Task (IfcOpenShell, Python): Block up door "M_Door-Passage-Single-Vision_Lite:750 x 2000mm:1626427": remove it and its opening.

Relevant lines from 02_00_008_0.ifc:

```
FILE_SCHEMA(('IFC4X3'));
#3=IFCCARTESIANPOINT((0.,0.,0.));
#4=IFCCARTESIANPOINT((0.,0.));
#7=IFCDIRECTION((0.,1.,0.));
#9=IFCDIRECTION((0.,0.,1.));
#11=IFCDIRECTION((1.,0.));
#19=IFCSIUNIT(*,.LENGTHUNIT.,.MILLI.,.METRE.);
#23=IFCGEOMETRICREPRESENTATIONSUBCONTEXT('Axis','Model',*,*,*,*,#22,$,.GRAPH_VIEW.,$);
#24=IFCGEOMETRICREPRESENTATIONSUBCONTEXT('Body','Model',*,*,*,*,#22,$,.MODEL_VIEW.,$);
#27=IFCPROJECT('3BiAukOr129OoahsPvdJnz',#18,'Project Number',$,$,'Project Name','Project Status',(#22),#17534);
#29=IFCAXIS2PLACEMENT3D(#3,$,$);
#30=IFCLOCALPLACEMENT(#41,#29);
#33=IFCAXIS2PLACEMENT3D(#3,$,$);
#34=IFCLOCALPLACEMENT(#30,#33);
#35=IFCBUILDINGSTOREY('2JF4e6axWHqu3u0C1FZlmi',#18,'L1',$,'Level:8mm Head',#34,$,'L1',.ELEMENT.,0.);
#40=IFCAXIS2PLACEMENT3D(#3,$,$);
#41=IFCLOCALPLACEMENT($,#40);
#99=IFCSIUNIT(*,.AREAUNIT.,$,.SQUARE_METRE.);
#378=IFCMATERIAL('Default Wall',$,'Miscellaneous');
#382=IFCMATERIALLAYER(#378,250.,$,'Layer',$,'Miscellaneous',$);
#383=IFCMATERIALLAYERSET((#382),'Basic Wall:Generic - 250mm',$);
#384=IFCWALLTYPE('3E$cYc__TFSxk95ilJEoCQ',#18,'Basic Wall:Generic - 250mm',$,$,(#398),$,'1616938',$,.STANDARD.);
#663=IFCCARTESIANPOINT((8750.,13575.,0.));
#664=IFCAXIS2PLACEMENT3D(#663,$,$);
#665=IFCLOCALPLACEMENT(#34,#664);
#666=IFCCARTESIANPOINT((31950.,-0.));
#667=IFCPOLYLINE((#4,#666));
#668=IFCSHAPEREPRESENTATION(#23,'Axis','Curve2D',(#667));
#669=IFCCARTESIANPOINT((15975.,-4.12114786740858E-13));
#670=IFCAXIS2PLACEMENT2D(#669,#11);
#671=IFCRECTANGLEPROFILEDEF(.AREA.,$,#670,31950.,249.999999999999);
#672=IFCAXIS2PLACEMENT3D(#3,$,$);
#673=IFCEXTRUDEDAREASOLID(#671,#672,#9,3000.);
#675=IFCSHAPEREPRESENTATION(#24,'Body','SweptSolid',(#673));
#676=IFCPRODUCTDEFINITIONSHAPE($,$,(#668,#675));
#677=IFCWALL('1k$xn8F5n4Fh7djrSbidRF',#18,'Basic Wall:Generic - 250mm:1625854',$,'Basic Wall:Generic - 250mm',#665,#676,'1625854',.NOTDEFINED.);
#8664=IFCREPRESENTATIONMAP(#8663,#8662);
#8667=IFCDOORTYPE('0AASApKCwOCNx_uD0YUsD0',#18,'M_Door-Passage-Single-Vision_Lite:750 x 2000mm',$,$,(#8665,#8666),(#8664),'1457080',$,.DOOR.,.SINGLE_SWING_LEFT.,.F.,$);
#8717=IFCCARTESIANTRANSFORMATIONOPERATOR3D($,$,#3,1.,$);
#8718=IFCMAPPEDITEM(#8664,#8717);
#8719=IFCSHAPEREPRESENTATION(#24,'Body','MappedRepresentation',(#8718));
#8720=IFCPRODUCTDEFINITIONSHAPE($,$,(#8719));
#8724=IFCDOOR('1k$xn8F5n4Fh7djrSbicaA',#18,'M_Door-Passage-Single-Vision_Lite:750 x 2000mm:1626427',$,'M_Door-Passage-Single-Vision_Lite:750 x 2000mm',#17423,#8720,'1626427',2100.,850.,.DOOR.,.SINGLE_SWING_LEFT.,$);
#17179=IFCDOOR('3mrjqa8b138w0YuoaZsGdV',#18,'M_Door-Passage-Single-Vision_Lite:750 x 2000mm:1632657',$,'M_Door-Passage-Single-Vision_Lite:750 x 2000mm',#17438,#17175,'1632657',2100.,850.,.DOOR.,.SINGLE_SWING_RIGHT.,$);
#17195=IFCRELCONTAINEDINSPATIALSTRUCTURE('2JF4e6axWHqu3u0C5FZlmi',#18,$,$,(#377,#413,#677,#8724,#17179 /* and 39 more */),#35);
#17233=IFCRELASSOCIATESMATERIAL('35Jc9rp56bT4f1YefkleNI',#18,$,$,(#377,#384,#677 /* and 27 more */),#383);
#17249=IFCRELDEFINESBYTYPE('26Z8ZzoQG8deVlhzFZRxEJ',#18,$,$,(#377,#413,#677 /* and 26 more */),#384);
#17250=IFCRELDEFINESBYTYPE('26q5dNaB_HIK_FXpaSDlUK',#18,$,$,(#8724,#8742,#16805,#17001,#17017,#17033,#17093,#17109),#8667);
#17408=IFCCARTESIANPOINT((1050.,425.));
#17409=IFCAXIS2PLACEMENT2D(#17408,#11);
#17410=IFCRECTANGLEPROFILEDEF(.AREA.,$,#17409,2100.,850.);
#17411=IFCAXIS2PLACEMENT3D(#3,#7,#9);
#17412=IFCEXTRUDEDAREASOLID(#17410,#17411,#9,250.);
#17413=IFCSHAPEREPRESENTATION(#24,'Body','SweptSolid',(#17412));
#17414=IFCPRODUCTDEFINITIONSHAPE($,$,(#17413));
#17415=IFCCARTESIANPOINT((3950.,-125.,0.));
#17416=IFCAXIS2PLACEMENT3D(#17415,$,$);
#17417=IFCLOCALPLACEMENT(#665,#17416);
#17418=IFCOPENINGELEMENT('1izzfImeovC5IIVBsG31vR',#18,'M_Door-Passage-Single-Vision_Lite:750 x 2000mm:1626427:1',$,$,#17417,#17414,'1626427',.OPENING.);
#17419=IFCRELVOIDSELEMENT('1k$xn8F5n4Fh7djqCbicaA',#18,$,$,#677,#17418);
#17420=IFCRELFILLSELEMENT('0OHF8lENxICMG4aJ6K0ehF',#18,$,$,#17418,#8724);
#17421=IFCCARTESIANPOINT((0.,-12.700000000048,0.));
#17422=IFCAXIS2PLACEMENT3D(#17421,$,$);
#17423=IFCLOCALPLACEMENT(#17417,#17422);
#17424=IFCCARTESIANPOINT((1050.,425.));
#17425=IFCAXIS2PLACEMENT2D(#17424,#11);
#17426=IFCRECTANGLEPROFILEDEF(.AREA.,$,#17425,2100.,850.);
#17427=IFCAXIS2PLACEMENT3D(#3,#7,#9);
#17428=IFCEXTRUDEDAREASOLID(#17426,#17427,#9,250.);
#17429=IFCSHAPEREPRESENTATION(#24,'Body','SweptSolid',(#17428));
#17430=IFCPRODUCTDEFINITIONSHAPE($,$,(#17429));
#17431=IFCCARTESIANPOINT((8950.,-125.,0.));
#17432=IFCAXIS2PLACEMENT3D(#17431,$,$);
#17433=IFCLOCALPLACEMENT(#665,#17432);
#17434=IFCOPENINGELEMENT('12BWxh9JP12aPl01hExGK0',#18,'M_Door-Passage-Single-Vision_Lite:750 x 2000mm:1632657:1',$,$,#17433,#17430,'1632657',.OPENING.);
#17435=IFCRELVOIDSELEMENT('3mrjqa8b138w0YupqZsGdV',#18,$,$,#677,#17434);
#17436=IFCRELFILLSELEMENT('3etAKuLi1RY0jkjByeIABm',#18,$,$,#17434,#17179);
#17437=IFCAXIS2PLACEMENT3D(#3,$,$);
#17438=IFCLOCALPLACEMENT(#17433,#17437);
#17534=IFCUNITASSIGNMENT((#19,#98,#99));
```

```python
import ifcopenshell
import ifcopenshell.api.feature
import ifcopenshell.api.root
import ifcopenshell.geom
import ifcopenshell.util.shape

model = ifcopenshell.open("02_00_008_0.ifc")
settings = ifcopenshell.geom.settings()


def volume(element):
    """Net volume in cubic metres, openings subtracted."""
    shape = ifcopenshell.geom.create_shape(settings, element)
    return ifcopenshell.util.shape.get_volume(shape.geometry)


door = model.by_guid("1k$xn8F5n4Fh7djrSbicaA")
opening = door.FillsVoids[0].RelatingOpeningElement
wall = opening.VoidsElements[0].RelatingBuildingElement
before = volume(wall)

ifcopenshell.api.root.remove_product(model, product=door)
ifcopenshell.api.feature.remove_feature(model, feature=opening)

after = volume(wall)

print(f"wall volume {before:.3f} -> {after:.3f} m3")

model.write("02_00_008_0_rev.ifc")
```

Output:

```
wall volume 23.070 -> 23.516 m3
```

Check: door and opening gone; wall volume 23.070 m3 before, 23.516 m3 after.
